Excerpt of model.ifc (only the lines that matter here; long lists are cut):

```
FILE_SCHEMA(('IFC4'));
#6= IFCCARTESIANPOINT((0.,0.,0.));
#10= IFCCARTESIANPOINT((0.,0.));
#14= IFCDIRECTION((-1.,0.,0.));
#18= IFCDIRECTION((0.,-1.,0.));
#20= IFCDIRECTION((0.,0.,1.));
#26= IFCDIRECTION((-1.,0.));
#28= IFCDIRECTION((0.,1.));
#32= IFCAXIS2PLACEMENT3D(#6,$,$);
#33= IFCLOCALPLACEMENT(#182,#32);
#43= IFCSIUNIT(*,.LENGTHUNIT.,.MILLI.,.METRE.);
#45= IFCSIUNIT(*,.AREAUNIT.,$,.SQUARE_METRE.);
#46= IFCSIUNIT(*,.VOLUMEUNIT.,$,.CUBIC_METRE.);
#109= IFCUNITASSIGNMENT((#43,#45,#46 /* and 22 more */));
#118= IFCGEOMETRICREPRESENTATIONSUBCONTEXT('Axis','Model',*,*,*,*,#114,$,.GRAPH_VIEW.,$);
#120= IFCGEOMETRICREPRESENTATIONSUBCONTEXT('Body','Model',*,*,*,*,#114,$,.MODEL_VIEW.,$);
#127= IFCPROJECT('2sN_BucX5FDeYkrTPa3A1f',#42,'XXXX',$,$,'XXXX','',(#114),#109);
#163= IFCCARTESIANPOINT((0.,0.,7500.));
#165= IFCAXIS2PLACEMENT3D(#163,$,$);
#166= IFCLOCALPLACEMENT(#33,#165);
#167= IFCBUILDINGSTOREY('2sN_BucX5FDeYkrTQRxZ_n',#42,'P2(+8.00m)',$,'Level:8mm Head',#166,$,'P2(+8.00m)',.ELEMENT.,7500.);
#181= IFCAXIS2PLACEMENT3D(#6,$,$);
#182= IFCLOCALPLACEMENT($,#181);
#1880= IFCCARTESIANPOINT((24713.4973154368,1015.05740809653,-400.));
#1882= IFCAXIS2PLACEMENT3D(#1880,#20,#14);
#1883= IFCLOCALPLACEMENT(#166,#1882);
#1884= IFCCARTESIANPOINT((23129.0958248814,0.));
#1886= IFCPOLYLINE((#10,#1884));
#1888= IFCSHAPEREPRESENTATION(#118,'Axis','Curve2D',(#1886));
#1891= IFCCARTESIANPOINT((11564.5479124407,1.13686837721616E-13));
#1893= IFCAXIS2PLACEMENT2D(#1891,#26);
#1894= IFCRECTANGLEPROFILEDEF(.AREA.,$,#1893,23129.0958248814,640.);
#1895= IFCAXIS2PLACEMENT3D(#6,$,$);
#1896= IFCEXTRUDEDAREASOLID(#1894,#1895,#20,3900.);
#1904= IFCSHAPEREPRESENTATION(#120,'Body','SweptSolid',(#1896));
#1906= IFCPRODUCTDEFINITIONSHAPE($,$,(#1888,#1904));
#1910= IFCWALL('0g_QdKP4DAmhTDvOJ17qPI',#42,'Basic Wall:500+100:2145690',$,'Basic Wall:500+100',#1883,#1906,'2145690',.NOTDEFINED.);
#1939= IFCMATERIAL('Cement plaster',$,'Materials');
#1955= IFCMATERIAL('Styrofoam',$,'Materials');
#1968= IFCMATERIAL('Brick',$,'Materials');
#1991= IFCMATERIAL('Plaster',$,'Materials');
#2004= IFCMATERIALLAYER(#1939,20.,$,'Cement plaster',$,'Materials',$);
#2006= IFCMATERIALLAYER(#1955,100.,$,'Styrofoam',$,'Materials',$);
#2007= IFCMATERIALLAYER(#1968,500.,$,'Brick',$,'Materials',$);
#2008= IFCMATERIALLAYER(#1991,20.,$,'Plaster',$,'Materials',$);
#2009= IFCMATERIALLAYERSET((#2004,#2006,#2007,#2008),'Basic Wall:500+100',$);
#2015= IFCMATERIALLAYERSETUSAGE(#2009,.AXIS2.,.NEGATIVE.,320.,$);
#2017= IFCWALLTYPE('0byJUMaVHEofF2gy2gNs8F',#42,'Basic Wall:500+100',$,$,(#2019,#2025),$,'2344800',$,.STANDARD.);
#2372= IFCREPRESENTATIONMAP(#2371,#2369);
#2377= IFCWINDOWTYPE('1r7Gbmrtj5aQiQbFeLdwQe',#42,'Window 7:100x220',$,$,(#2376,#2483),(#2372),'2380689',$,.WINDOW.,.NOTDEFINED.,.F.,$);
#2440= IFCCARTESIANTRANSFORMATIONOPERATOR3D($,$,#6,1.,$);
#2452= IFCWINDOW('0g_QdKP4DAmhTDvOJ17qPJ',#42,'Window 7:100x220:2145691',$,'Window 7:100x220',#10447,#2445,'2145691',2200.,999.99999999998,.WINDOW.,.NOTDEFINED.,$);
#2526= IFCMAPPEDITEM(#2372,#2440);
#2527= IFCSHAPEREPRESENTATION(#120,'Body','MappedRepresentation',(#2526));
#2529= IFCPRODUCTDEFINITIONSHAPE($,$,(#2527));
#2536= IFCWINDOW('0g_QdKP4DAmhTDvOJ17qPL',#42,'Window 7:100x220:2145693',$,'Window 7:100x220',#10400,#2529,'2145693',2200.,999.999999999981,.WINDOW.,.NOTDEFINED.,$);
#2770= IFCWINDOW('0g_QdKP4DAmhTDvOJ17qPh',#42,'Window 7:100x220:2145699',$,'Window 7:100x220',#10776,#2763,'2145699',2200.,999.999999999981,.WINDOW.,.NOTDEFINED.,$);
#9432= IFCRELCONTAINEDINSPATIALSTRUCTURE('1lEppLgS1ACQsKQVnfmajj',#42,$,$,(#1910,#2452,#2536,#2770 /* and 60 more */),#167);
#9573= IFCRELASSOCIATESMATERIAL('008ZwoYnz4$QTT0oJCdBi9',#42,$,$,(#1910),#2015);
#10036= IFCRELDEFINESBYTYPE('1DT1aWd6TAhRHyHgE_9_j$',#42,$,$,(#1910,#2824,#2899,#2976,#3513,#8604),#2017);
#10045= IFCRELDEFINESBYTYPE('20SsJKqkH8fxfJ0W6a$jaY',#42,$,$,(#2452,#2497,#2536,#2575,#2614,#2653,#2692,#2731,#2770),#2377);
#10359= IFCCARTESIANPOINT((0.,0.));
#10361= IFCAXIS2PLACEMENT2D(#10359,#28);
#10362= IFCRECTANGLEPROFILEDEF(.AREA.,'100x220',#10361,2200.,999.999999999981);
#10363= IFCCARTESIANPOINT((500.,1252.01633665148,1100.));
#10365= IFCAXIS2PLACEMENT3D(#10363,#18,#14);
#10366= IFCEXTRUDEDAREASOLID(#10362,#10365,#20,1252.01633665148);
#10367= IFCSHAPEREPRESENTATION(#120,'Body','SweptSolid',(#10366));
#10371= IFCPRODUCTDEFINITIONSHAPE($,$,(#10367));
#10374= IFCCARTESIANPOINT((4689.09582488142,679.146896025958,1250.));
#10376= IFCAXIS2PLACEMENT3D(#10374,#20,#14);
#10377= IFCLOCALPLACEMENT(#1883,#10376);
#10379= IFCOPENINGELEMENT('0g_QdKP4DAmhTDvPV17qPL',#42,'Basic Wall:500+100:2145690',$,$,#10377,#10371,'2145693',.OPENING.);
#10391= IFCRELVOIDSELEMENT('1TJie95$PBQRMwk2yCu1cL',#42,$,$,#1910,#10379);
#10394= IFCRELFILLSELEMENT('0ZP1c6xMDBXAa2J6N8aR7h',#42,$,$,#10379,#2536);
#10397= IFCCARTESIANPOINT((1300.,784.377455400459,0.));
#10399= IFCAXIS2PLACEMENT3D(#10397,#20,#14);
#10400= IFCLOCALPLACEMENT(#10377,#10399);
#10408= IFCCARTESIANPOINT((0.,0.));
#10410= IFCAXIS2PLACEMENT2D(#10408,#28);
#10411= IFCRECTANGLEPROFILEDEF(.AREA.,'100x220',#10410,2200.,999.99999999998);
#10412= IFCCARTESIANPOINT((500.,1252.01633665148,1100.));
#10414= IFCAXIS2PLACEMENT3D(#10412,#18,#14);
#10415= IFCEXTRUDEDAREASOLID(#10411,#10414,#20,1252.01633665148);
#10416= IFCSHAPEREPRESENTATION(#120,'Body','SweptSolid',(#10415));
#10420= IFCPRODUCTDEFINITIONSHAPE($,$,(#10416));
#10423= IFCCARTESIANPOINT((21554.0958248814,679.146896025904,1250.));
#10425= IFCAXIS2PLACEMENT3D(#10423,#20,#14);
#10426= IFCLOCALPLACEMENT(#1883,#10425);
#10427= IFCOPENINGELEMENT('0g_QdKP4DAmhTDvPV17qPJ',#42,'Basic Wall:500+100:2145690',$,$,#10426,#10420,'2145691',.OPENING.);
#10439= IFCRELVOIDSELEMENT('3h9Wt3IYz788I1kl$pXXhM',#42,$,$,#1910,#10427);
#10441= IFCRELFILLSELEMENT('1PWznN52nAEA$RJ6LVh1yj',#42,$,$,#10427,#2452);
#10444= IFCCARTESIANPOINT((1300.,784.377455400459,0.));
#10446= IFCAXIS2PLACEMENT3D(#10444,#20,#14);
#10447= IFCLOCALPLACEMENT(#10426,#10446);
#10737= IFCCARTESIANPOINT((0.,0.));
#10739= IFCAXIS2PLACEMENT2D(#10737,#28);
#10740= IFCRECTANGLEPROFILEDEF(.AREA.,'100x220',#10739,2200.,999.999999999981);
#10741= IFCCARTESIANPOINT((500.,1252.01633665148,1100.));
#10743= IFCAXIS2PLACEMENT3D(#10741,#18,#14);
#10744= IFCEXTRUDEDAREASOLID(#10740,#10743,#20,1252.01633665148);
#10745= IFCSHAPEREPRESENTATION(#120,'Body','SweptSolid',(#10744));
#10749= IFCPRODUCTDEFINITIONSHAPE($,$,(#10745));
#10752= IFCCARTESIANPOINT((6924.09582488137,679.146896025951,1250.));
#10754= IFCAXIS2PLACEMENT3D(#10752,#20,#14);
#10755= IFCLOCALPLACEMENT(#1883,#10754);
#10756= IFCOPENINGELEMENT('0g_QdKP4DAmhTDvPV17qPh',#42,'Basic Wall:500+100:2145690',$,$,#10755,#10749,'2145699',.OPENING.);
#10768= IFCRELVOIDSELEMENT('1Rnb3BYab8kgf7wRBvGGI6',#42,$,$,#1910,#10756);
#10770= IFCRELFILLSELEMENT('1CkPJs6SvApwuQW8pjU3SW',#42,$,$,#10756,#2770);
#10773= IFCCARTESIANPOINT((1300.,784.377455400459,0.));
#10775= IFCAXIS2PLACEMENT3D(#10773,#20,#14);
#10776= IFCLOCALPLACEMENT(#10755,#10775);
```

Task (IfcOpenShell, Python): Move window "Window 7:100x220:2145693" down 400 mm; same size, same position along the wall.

```python
import numpy as np
import ifcopenshell
import ifcopenshell.api.geometry
import ifcopenshell.util.placement
import ifcopenshell.util.unit

model = ifcopenshell.open("model.ifc")
unit_scale = ifcopenshell.util.unit.calculate_unit_scale(model)

window = model.by_guid("0g_QdKP4DAmhTDvOJ17qPL")
opening = window.FillsVoids[0].RelatingOpeningElement
dz = -400.0

shift = np.array([0.0, 0.0, dz])
# The window is placed relative to its opening, so it follows when the opening moves.
matrix = ifcopenshell.util.placement.get_local_placement(opening.ObjectPlacement)
matrix[:3, 3] += shift
ifcopenshell.api.geometry.edit_object_placement(
    model, product=opening, matrix=matrix, is_si=False, should_transform_children=True
)

print(f"moved by {dz * unit_scale:+.3f} m")

model.write("model_rev.ifc")
```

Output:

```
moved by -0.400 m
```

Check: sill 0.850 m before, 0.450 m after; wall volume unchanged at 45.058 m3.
